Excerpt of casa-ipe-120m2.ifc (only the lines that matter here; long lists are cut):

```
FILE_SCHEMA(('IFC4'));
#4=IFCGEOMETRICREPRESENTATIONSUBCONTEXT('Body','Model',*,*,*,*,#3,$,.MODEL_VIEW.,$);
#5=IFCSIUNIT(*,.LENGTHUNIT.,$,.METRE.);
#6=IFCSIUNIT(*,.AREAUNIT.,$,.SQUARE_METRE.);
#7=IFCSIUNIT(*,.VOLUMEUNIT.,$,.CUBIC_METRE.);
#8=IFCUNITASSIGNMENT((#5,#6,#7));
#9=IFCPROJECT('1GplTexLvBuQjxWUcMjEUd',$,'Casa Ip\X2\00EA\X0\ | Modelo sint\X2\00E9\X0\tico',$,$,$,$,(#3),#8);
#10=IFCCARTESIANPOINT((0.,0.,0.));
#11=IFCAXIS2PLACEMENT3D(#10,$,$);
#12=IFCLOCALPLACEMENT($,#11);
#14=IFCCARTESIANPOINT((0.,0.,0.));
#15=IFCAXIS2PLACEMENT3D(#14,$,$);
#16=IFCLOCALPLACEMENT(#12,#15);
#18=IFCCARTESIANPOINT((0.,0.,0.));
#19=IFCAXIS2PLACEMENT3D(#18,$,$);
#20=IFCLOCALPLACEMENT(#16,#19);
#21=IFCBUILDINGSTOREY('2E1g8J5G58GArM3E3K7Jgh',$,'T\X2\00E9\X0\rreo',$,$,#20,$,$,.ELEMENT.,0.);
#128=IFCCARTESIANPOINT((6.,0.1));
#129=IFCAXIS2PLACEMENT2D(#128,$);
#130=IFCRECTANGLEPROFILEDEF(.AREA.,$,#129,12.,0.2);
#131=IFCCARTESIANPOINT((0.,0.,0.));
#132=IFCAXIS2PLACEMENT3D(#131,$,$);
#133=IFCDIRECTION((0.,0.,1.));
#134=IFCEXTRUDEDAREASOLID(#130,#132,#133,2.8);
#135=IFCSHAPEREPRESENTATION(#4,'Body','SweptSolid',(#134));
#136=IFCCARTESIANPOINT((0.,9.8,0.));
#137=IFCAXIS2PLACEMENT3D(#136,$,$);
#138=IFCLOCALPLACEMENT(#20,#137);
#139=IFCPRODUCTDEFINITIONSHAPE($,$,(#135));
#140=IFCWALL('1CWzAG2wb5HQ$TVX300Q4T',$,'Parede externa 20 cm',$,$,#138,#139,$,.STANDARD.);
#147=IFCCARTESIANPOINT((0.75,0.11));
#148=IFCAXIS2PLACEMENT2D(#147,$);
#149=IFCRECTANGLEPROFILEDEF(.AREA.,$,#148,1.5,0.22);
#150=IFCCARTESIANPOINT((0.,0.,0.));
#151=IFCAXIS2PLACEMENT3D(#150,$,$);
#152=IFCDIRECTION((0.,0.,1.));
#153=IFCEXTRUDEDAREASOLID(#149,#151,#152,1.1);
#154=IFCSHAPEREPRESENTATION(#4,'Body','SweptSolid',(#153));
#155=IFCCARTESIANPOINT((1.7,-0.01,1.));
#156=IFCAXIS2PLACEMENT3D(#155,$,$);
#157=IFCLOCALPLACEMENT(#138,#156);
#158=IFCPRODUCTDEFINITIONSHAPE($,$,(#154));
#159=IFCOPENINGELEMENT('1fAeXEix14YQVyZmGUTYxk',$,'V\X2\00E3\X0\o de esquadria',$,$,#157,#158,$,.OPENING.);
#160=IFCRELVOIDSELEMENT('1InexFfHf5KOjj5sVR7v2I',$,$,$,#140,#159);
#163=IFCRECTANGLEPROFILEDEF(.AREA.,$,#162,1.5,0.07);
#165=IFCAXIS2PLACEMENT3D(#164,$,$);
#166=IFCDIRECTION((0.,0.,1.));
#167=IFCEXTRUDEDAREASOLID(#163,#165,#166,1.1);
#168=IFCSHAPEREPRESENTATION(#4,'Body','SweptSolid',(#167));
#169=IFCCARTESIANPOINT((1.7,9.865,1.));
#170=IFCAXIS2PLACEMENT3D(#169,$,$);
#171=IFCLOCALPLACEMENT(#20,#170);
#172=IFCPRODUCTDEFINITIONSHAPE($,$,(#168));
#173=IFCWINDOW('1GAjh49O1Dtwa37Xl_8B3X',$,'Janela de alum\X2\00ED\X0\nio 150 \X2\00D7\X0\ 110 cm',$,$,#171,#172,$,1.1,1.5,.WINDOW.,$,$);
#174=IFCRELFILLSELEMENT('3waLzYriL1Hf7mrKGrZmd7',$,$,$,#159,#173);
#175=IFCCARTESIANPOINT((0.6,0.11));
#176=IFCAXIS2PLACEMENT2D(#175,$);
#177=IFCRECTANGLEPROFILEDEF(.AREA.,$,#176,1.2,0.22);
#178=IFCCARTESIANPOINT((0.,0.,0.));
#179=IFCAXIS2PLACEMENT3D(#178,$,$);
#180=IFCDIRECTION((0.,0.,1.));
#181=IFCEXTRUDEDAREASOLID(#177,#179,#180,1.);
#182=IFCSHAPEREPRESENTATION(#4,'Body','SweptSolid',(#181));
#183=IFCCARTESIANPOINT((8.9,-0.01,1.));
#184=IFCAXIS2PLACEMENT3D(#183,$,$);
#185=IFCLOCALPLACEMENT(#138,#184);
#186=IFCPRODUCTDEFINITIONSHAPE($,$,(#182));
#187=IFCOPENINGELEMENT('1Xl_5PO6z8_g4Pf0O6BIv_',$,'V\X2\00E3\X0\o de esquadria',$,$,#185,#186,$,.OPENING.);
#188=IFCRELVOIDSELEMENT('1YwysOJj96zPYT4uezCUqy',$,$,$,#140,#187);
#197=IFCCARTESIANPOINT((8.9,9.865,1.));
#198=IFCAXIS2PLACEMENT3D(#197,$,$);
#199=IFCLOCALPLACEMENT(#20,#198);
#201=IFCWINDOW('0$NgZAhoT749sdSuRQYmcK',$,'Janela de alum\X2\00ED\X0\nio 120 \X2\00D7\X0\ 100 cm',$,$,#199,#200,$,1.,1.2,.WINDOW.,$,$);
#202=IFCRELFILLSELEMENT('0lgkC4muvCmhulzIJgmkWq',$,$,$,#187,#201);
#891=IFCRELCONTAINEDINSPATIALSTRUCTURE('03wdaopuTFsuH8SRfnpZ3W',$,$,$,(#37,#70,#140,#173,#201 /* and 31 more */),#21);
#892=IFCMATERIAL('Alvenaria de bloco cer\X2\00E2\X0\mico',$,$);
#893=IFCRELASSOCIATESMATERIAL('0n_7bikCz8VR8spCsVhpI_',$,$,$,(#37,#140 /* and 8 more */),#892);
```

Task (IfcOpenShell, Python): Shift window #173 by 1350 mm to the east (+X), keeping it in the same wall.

```python
import ifcopenshell
import ifcopenshell.api.geometry
import ifcopenshell.util.placement
import ifcopenshell.util.unit

model = ifcopenshell.open("casa-ipe-120m2.ifc")
unit_scale = ifcopenshell.util.unit.calculate_unit_scale(model)

window = model.by_id(173)
opening = window.FillsVoids[0].RelatingOpeningElement
wall = opening.VoidsElements[0].RelatingBuildingElement

wall_matrix = ifcopenshell.util.placement.get_local_placement(wall.ObjectPlacement)
shift = wall_matrix[:3, 0] * 1.35 / unit_scale
before = ifcopenshell.util.placement.get_local_placement(window.ObjectPlacement)[:3, 3].copy()

# The window is not placed relative to its opening, so move both.
for product in (opening, window):
    matrix = ifcopenshell.util.placement.get_local_placement(product.ObjectPlacement)
    matrix[:3, 3] += shift
    ifcopenshell.api.geometry.edit_object_placement(model, product=product, matrix=matrix, is_si=False)

after = ifcopenshell.util.placement.get_local_placement(window.ObjectPlacement)[:3, 3]
print("window moved by", (after - before).round(3) + 0.0)

model.write("casa-ipe-120m2_rev.ifc")
```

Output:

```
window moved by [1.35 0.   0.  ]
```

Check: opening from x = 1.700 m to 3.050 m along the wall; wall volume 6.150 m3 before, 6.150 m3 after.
